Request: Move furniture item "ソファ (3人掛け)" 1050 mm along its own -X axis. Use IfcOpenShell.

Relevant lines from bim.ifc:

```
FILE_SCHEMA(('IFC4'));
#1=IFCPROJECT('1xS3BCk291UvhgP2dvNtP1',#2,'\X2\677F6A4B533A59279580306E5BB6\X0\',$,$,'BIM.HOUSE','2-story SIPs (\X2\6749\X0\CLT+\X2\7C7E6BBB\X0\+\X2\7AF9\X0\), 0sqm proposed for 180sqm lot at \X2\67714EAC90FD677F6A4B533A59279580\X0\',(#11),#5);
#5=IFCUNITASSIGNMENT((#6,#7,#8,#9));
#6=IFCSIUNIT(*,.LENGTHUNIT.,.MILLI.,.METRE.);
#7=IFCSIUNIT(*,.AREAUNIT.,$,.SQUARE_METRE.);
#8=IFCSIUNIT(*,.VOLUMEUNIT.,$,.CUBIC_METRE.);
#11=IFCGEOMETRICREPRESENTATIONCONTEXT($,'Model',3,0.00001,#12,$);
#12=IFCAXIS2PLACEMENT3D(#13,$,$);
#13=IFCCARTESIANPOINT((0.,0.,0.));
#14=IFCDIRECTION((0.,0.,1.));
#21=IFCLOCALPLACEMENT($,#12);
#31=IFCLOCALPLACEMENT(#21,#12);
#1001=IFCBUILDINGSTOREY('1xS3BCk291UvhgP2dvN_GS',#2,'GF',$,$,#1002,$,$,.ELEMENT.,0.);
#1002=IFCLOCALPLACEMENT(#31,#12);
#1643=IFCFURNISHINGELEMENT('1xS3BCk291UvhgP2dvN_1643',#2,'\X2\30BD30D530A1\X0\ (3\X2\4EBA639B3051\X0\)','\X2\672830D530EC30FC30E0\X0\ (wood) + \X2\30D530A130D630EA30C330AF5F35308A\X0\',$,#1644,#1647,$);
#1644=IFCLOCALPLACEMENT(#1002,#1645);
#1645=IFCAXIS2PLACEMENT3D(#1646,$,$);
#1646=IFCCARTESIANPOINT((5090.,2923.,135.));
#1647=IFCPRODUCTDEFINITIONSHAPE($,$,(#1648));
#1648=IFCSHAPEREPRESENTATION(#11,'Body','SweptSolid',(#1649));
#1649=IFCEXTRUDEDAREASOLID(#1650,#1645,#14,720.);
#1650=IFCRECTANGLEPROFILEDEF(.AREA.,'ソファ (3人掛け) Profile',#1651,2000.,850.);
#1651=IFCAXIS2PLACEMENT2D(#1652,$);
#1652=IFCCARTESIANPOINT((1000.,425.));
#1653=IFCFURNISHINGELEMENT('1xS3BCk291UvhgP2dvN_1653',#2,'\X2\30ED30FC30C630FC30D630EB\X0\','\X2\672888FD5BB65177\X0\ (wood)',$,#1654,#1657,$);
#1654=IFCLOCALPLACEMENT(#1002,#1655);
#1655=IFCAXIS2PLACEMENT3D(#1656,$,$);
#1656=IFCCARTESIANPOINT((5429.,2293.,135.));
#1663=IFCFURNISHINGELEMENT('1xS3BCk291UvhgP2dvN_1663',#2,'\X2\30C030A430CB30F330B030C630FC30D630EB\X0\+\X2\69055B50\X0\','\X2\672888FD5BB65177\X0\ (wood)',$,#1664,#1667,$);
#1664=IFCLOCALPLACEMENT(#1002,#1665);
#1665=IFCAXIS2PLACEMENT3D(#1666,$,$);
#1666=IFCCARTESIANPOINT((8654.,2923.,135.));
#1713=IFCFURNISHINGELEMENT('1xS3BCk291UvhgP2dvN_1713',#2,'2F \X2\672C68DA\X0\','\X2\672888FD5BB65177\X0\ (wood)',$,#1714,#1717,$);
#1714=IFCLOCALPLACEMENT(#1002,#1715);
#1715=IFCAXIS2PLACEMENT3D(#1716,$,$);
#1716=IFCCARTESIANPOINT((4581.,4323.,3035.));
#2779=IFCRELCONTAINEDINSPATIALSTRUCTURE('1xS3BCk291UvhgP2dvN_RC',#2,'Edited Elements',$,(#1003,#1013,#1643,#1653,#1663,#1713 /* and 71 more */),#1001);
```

```python
import ifcopenshell
import ifcopenshell.api.geometry
import ifcopenshell.util.placement
import ifcopenshell.util.unit

model = ifcopenshell.open("bim.ifc")
unit_scale = ifcopenshell.util.unit.calculate_unit_scale(model)

item = model.by_id(1643)
matrix = ifcopenshell.util.placement.get_local_placement(item.ObjectPlacement)
matrix[:3, 3] -= matrix[:3, 0] * 1.05 / unit_scale
ifcopenshell.api.geometry.edit_object_placement(model, product=item, matrix=matrix, is_si=False)

print(ifcopenshell.util.placement.get_local_placement(item.ObjectPlacement).round(3) + 0.0)

model.write("bim_rev.ifc")
```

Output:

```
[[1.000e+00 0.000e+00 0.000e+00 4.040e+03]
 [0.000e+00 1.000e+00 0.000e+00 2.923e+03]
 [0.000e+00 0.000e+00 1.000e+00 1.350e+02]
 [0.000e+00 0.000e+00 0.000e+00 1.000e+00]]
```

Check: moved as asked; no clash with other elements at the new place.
